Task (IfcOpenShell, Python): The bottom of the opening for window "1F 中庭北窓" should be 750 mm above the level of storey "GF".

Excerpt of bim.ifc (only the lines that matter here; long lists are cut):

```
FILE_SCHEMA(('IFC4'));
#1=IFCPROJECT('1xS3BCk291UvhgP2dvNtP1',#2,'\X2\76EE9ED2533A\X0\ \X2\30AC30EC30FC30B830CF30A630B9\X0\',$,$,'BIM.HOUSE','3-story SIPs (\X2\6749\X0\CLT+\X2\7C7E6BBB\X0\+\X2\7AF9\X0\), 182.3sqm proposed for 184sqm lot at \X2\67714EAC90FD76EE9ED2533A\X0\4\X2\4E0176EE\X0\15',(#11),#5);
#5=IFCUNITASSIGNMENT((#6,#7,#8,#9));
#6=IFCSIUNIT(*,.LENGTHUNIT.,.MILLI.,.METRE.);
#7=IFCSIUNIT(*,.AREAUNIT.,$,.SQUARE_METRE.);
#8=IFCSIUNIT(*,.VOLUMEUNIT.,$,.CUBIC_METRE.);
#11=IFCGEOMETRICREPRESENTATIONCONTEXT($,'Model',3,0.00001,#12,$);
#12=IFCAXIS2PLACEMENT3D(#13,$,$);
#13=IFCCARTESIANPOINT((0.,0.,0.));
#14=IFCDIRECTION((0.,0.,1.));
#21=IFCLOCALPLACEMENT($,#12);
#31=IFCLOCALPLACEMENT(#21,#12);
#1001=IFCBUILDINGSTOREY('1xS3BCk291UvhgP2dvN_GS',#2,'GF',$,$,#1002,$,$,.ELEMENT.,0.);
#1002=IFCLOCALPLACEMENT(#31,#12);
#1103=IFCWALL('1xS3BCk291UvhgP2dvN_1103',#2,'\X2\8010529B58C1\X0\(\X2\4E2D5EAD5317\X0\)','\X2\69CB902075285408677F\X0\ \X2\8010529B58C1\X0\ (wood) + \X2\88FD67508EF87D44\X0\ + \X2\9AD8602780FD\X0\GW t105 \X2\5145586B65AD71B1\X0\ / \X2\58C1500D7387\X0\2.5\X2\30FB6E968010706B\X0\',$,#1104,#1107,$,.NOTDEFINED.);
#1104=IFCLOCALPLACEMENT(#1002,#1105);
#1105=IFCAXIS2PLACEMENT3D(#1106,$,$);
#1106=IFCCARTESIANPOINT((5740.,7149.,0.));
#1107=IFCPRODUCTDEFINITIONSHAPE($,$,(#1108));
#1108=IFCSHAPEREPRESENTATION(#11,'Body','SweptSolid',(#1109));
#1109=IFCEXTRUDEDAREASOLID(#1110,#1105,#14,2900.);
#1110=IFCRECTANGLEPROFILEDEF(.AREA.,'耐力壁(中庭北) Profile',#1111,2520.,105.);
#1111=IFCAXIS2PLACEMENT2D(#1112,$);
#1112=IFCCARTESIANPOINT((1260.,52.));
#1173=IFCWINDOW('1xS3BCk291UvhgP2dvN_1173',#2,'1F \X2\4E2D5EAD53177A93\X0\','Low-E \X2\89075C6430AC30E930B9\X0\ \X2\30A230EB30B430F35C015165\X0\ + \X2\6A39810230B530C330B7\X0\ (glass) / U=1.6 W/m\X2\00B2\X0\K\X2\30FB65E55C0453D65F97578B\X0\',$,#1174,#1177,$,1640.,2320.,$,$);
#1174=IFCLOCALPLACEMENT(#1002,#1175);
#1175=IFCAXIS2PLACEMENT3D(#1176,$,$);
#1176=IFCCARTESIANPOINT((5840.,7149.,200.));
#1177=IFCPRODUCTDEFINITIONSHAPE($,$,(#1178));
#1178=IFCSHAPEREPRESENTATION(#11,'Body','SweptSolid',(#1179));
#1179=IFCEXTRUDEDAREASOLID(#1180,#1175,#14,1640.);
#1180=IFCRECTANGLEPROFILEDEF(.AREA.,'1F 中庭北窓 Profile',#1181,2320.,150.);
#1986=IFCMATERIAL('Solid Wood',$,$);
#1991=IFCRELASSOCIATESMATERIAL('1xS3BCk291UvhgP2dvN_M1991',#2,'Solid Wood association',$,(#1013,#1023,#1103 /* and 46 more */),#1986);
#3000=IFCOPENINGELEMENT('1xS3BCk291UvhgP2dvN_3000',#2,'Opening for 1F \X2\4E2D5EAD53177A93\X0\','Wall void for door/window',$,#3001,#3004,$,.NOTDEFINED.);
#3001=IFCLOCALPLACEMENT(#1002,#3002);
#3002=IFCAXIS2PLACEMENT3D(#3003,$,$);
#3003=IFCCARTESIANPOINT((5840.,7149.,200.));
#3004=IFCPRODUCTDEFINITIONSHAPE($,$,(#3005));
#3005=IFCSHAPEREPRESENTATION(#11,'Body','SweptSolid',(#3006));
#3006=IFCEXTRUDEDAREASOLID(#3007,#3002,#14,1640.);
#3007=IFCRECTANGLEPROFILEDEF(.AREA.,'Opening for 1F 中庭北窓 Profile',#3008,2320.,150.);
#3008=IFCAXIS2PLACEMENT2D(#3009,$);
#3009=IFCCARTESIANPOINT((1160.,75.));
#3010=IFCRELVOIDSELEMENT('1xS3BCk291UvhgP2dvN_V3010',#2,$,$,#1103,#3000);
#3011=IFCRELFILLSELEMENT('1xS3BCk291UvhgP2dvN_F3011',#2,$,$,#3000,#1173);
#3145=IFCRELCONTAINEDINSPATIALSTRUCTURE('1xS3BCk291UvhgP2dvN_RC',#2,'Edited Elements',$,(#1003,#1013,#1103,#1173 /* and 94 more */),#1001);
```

```python
import numpy as np
import ifcopenshell
import ifcopenshell.api.geometry
import ifcopenshell.geom
import ifcopenshell.util.element
import ifcopenshell.util.placement
import ifcopenshell.util.shape
import ifcopenshell.util.unit

model = ifcopenshell.open("bim.ifc")
unit_scale = ifcopenshell.util.unit.calculate_unit_scale(model)

window = model.by_guid("1xS3BCk291UvhgP2dvN_1173")
opening = window.FillsVoids[0].RelatingOpeningElement
storey = ifcopenshell.util.element.get_container(window, ifc_class="IfcBuildingStorey")
level = ifcopenshell.util.placement.get_local_placement(storey.ObjectPlacement)[2, 3]

# The opening's origin need not be at the sill, so measure its lowest point.
shape = ifcopenshell.geom.create_shape(ifcopenshell.geom.settings(), opening)
bottom = ifcopenshell.util.shape.get_shape_bottom_elevation(shape, shape.geometry) / unit_scale
dz = level + 0.75 / unit_scale - bottom

shift = np.array([0.0, 0.0, dz])
# The window is not placed relative to its opening, so move both.
for product in (opening, window):
    matrix = ifcopenshell.util.placement.get_local_placement(product.ObjectPlacement)
    matrix[:3, 3] += shift
    ifcopenshell.api.geometry.edit_object_placement(model, product=product, matrix=matrix, is_si=False)

print(f"moved by {dz * unit_scale:+.3f} m")

model.write("bim_v2.ifc")
```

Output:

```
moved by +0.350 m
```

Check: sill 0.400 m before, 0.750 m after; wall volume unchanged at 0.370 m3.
